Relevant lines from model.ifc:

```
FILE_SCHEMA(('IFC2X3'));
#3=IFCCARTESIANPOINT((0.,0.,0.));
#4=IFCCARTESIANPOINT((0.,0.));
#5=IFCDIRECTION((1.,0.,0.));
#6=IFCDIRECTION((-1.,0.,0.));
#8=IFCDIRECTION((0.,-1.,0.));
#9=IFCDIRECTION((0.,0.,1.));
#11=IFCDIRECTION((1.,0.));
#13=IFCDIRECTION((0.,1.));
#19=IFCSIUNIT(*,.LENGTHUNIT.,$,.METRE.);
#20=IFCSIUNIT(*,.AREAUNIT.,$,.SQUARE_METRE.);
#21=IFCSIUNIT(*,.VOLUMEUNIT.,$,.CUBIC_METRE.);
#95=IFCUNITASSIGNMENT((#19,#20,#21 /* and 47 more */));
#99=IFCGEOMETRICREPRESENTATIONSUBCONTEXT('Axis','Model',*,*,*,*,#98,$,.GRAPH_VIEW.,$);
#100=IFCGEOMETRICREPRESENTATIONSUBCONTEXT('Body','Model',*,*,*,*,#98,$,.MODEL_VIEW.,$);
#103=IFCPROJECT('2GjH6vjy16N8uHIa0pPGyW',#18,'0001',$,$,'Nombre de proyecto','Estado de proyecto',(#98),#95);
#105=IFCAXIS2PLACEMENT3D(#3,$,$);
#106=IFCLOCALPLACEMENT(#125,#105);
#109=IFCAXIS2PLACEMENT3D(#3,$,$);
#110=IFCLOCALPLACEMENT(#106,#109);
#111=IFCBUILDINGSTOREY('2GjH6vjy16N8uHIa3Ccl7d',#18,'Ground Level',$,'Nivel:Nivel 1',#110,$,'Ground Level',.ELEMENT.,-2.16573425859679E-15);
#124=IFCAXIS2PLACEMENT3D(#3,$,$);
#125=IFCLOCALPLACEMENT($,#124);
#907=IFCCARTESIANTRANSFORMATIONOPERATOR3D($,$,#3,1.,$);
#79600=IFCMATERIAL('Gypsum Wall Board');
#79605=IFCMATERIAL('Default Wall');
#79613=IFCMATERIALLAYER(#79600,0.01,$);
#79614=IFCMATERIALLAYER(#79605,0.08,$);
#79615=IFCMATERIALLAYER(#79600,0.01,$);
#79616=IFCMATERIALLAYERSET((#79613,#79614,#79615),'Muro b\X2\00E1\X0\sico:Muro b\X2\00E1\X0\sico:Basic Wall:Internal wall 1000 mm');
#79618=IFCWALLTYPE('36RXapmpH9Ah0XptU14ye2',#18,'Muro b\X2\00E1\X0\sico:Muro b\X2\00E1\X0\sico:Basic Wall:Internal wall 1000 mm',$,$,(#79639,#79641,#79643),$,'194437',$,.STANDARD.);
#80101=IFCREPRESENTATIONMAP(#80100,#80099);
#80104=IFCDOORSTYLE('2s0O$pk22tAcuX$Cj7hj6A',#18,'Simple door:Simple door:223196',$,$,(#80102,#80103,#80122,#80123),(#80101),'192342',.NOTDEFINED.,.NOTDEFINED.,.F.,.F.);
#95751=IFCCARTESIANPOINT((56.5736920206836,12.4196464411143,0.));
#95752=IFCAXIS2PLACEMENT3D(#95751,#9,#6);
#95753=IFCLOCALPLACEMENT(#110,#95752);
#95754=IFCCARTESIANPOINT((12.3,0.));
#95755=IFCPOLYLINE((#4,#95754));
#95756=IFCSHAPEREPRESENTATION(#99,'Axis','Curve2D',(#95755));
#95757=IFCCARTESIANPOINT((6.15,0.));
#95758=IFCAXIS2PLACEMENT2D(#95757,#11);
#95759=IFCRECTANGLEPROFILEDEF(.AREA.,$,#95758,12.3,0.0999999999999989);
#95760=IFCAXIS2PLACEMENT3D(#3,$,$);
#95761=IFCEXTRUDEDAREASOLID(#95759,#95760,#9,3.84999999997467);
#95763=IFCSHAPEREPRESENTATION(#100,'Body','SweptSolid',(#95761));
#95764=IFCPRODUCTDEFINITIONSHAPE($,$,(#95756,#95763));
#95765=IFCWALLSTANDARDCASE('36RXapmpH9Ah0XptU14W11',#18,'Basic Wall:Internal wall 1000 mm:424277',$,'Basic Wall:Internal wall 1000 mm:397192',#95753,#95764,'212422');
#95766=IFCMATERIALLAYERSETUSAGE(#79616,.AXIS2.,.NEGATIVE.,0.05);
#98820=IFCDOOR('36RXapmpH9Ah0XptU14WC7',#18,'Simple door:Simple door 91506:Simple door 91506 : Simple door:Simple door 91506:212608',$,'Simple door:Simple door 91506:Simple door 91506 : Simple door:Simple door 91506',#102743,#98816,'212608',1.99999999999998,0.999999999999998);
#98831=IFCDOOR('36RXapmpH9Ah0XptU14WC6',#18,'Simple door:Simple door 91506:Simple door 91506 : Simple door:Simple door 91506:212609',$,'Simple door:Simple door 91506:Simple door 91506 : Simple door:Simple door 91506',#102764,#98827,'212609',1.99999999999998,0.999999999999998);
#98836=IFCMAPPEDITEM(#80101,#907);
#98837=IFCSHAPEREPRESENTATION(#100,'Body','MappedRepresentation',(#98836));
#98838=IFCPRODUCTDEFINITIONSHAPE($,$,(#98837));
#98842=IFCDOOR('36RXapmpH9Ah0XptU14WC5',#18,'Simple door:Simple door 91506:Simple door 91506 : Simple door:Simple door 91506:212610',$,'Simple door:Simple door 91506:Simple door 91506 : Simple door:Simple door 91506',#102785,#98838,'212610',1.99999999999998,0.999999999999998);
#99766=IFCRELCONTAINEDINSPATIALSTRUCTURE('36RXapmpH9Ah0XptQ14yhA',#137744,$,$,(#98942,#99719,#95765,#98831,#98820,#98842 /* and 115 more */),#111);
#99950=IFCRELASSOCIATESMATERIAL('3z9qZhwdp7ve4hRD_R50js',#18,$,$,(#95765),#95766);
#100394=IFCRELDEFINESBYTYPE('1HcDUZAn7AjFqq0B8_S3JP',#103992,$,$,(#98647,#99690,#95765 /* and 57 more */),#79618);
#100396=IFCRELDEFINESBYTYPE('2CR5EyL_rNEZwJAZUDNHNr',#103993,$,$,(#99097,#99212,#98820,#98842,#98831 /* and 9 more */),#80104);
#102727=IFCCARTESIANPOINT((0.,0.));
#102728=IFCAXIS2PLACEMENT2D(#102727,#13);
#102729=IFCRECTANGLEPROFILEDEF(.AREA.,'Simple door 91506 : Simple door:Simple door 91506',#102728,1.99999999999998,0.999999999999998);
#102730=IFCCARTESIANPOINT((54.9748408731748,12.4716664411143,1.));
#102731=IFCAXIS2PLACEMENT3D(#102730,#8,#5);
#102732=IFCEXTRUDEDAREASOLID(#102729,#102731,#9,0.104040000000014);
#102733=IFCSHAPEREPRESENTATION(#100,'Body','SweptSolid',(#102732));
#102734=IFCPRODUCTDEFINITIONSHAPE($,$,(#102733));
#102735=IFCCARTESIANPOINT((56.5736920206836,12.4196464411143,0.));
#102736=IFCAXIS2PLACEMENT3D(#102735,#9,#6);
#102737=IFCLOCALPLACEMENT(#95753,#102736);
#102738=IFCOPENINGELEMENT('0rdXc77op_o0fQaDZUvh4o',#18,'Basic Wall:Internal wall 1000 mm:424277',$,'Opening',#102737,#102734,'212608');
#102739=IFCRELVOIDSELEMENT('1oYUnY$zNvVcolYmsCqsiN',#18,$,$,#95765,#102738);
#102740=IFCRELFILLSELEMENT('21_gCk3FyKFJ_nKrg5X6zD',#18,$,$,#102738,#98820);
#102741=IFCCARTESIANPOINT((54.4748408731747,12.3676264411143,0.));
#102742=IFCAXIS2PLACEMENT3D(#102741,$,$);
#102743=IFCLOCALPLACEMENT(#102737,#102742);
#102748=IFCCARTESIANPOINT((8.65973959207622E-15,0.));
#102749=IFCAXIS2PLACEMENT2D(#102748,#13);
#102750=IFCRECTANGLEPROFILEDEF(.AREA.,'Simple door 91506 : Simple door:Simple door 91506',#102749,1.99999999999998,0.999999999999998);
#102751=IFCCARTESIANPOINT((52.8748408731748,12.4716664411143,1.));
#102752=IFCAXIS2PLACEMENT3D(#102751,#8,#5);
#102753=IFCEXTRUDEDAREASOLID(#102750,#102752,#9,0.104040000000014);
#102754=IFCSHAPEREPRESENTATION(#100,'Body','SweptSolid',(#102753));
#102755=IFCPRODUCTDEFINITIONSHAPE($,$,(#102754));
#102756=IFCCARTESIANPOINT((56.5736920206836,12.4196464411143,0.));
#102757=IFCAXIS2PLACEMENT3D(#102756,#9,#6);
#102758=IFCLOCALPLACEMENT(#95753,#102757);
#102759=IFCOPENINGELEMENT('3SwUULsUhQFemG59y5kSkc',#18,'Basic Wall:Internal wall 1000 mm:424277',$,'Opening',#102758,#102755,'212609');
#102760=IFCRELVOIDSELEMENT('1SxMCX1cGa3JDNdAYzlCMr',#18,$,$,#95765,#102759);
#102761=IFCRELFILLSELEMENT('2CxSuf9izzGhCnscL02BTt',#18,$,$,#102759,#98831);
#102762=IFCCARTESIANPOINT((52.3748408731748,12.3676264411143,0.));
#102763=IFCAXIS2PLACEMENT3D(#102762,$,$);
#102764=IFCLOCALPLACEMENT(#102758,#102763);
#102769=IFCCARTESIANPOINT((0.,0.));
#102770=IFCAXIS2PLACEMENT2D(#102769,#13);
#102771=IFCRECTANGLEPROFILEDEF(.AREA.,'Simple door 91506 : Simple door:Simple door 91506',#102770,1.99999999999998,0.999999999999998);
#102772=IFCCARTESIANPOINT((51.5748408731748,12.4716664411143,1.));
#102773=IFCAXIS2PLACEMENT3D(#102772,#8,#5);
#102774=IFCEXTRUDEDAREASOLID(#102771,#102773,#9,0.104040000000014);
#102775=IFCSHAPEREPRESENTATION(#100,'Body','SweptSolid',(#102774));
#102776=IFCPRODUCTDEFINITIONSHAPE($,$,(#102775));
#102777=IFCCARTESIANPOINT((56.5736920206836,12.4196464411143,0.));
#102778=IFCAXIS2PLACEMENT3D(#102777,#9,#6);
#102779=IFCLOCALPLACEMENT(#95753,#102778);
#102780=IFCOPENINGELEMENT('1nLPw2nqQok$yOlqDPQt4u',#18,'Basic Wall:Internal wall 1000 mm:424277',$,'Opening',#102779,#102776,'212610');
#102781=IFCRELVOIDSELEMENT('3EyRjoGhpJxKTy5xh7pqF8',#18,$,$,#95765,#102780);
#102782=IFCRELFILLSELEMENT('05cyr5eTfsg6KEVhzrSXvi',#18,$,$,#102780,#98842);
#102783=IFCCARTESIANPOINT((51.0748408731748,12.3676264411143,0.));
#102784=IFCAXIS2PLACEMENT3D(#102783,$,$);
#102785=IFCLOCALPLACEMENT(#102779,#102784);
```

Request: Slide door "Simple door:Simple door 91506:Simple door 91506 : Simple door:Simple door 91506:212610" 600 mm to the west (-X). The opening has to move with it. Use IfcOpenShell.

```python
import ifcopenshell
import ifcopenshell.api.geometry
import ifcopenshell.util.placement
import ifcopenshell.util.unit

model = ifcopenshell.open("model.ifc")
unit_scale = ifcopenshell.util.unit.calculate_unit_scale(model)

door = model.by_id(98842)
opening = door.FillsVoids[0].RelatingOpeningElement
wall = opening.VoidsElements[0].RelatingBuildingElement

wall_matrix = ifcopenshell.util.placement.get_local_placement(wall.ObjectPlacement)
shift = wall_matrix[:3, 0] * 0.6 / unit_scale
before = ifcopenshell.util.placement.get_local_placement(door.ObjectPlacement)[:3, 3].copy()

# The door is placed relative to its opening, so it follows when the opening moves.
matrix = ifcopenshell.util.placement.get_local_placement(opening.ObjectPlacement)
matrix[:3, 3] += shift
ifcopenshell.api.geometry.edit_object_placement(
    model, product=opening, matrix=matrix, is_si=False, should_transform_children=True
)

after = ifcopenshell.util.placement.get_local_placement(door.ObjectPlacement)[:3, 3]
print("door moved by", (after - before).round(3) + 0.0)

model.write("model_updated.ifc")
```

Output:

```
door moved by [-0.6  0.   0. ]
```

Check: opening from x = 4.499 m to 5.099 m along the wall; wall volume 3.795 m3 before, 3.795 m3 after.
